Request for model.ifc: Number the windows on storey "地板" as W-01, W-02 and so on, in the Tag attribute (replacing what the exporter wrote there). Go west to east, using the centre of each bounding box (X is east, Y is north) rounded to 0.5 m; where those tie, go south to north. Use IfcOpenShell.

First a look at what the model holds.

```python
import ifcopenshell
import ifcopenshell.util.element
import ifcopenshell.util.placement

model = ifcopenshell.open("model.ifc")
print(model.schema)
storey = next(s for s in model.by_type("IfcBuildingStorey") if s.Name == "地板")
windows = [e for e in ifcopenshell.util.element.get_decomposition(storey) if e.is_a("IfcWindow")]
for e in sorted(windows, key=lambda e: e.id()):
    origin = ifcopenshell.util.placement.get_local_placement(e.ObjectPlacement)[:3, 3]
    print(e.id(), e.Tag, e.Name, origin.round(2) + 0.0, sep=" | ")
```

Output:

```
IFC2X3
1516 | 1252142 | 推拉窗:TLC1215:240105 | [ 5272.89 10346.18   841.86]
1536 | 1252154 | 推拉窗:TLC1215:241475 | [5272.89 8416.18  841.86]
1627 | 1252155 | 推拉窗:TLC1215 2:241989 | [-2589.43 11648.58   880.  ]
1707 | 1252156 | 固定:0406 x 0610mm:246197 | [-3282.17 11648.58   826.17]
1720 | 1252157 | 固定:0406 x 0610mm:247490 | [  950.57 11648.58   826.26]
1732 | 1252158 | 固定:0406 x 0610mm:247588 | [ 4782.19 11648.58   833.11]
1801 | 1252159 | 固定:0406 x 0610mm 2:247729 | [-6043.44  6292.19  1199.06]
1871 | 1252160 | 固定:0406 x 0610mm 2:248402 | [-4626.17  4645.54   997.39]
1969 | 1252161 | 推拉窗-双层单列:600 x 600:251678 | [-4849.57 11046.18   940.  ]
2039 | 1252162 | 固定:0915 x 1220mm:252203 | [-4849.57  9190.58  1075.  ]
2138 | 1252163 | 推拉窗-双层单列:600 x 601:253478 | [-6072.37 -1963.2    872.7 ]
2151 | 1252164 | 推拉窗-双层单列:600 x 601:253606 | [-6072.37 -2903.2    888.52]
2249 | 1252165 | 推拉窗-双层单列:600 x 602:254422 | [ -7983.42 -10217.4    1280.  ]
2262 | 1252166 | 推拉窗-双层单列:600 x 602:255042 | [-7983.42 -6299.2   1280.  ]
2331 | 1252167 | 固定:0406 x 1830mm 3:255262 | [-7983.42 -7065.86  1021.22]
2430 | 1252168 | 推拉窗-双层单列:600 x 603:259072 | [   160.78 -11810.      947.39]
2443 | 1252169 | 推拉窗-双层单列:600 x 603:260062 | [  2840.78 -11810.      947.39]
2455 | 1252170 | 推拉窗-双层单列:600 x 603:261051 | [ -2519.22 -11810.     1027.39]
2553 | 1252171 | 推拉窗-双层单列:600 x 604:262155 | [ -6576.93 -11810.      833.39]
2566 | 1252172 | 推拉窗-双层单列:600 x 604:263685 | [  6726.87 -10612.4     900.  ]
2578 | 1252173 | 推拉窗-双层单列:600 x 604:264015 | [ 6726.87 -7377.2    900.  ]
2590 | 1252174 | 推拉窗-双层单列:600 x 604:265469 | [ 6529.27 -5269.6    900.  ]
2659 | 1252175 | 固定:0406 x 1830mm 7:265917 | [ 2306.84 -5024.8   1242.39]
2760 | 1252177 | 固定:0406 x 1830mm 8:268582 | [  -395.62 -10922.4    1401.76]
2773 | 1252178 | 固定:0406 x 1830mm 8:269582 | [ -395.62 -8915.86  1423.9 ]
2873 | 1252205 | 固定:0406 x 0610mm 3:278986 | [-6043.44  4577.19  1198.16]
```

```python
import ifcopenshell
import ifcopenshell.geom
import ifcopenshell.util.element
import ifcopenshell.util.shape

model = ifcopenshell.open("model.ifc")
settings = ifcopenshell.geom.settings()
settings.set("use-world-coords", True)


def centre(element):
    shape = ifcopenshell.geom.create_shape(settings, element)
    return ifcopenshell.util.shape.get_bbox_centroid(shape.geometry)


storey = next(s for s in model.by_type("IfcBuildingStorey") if s.Name == "地板")
windows = [e for e in ifcopenshell.util.element.get_decomposition(storey) if e.is_a("IfcWindow")]

# Insertion points can sit at a corner or the storey origin, so sort by the geometry (in metres).
centres = {e: centre(e) for e in windows}
windows.sort(key=lambda e: (round(centres[e][0] / 0.5), centres[e][1]))

for i, e in enumerate(windows, start=1):
    number = f"W-{i:02d}"
    e.Tag = number
    print(e.id(), number)

model.write("model-out.ifc")
```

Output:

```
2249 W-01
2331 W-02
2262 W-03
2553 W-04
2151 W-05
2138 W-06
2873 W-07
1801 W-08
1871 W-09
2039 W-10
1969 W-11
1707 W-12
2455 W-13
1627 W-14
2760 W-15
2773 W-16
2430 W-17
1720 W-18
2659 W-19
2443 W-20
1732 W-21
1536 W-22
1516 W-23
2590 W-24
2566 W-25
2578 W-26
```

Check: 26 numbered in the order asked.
